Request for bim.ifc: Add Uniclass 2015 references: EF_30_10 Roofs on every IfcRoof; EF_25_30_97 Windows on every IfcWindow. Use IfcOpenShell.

First a look at what the model holds.

```python
import ifcopenshell

model = ifcopenshell.open("bim.ifc")
print(model.schema)
print("classifications:", [c.Name for c in model.by_type("IfcClassification")])
for ifc_class in ("IfcDoor", "IfcRoof", "IfcStair", "IfcWall", "IfcWindow"):
    print(ifc_class, len(model.by_type(ifc_class)))
```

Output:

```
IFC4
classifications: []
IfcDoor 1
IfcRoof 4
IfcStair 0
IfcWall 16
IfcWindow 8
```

```python
import ifcopenshell
import ifcopenshell.api.classification

model = ifcopenshell.open("bim.ifc")

system = ifcopenshell.api.classification.add_classification(model, classification="Uniclass 2015")

codes = {
    "IfcRoof": ("EF_30_10", "Roofs"),
    "IfcWindow": ("EF_25_30_97", "Windows"),
}
for ifc_class, (code, name) in codes.items():
    products = model.by_type(ifc_class)
    ifcopenshell.api.classification.add_reference(
        model, products=products, classification=system, identification=code, name=name
    )
    print(code, len(products))

model.write("bim_v2.ifc")
```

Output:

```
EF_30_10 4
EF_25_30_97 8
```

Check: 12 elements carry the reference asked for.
